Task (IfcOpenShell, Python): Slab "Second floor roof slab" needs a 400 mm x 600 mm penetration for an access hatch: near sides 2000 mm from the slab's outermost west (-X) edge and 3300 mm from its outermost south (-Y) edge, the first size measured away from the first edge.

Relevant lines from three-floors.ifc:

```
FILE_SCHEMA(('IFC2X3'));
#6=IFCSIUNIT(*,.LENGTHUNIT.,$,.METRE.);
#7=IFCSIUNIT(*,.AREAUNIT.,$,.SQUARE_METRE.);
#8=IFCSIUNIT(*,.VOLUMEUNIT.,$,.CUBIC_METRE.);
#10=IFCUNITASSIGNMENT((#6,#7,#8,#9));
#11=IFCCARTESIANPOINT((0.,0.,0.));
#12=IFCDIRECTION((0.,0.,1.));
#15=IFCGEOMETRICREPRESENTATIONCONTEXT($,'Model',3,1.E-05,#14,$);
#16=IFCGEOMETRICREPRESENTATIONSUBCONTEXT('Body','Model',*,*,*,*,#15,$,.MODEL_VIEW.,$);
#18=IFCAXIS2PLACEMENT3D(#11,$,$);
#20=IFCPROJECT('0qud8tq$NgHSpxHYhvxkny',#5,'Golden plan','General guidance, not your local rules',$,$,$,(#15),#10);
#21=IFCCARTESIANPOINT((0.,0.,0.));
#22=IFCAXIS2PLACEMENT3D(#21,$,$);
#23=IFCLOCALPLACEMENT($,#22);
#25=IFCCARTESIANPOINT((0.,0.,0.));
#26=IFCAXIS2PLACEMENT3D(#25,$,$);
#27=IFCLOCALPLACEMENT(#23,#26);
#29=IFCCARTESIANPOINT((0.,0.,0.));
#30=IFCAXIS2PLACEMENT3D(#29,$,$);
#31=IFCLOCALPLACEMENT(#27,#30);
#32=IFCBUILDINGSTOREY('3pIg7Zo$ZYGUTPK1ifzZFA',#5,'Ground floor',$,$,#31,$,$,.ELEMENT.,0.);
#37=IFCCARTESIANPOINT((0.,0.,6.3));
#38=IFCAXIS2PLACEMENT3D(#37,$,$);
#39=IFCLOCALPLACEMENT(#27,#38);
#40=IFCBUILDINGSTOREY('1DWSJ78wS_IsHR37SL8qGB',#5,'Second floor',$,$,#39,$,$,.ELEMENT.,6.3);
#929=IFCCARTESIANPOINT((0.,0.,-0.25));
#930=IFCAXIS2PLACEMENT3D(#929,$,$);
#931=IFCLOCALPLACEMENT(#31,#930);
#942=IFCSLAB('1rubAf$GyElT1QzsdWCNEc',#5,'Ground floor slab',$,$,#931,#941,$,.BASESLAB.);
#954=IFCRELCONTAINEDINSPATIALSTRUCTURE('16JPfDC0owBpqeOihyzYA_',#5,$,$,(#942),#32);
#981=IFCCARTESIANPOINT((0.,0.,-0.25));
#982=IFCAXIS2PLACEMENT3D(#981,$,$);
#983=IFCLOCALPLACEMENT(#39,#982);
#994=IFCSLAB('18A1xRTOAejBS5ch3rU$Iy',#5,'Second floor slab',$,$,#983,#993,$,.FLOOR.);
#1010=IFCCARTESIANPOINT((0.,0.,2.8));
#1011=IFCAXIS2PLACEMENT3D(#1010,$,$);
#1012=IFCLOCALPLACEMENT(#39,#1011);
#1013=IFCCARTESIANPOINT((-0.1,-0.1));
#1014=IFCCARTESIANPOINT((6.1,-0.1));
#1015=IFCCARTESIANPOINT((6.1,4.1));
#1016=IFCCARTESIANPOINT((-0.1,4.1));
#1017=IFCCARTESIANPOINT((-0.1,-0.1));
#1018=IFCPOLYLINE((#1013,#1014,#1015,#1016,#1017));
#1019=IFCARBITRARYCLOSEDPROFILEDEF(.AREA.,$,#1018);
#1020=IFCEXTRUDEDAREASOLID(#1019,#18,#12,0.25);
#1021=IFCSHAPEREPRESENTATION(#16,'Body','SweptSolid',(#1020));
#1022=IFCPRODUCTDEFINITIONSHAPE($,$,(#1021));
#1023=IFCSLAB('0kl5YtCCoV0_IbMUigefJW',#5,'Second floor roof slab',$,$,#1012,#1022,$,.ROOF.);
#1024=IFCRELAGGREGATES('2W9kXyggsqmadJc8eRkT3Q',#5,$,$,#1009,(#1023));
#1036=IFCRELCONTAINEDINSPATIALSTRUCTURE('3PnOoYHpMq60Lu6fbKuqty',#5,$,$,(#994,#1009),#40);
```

```python
import numpy as np
import ifcopenshell
import ifcopenshell.api.feature
import ifcopenshell.api.geometry
import ifcopenshell.api.root
import ifcopenshell.geom
import ifcopenshell.util.placement
import ifcopenshell.util.representation
import ifcopenshell.util.shape
import ifcopenshell.util.unit

model = ifcopenshell.open("three-floors.ifc")
unit_scale = ifcopenshell.util.unit.calculate_unit_scale(model)
settings = ifcopenshell.geom.settings()


def volume(element):
    """Net volume in cubic metres, openings subtracted."""
    shape = ifcopenshell.geom.create_shape(settings, element)
    return ifcopenshell.util.shape.get_volume(shape.geometry)


slab = model.by_guid("0kl5YtCCoV0_IbMUigefJW")
before = volume(slab)

# Extent in the slab's own axes, in metres. The edges named are its -X and -Y sides.
slab_shape = ifcopenshell.geom.create_shape(settings, slab)
vertices = ifcopenshell.util.shape.get_vertices(slab_shape.geometry)
x_min, y_min, bottom = vertices.min(axis=0)
top = vertices[:, 2].max()

opening = ifcopenshell.api.root.create_entity(model, ifc_class="IfcOpeningElement", name="Access hatch opening")
context = ifcopenshell.util.representation.get_context(model, "Model", "Body", "MODEL_VIEW")
width, depth = 0.4, 0.6
outline = [(0.0, 0.0), (width, 0.0), (width, depth), (0.0, depth), (0.0, 0.0)]
# Overshoot both faces by 50 mm so the cut is clean.
shape = ifcopenshell.api.geometry.add_slab_representation(
    model, context=context, depth=top - bottom + 0.1, polyline=outline
)
ifcopenshell.api.geometry.assign_representation(model, product=opening, representation=shape)

matrix = ifcopenshell.util.placement.get_local_placement(slab.ObjectPlacement)
matrix[:, 3] = matrix @ np.append(np.array([x_min + 2, y_min + 3.3, bottom - 0.05]) / unit_scale, 1.0)
ifcopenshell.api.geometry.edit_object_placement(model, product=opening, matrix=matrix, is_si=False)
ifcopenshell.api.feature.add_feature(model, feature=opening, element=slab)

after = volume(slab)

print(f"slab volume {before:.3f} -> {after:.3f} m3")

model.write("three-floors-out.ifc")
```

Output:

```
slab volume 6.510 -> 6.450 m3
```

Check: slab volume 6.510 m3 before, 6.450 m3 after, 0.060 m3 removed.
